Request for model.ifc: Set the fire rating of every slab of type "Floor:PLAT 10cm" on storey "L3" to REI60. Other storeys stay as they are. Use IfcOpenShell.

First a look at what the model holds.

```python
import ifcopenshell
import ifcopenshell.util.element

model = ifcopenshell.open("model.ifc")
print(model.schema)
storey = next(s for s in model.by_type("IfcBuildingStorey") if s.Name == "L3")
slabs = [e for e in ifcopenshell.util.element.get_decomposition(storey) if e.is_a("IfcSlab")]
seen = {}
for e in slabs:
    element_type = ifcopenshell.util.element.get_type(e)
    key = (element_type.Name if element_type != e and element_type else None, ifcopenshell.util.element.get_pset(e, "Pset_SlabCommon", "FireRating"))
    seen[key] = seen.get(key, 0) + 1
for (name, value), count in sorted(seen.items(), key=str):
    print(count, "x", name, "|", value)
```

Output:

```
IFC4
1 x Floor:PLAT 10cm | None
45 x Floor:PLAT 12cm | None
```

```python
import ifcopenshell
import ifcopenshell.api.pset
import ifcopenshell.util.element

model = ifcopenshell.open("model.ifc")

storey = next(s for s in model.by_type("IfcBuildingStorey") if s.Name == "L3")
slabs = [e for e in ifcopenshell.util.element.get_decomposition(storey) if e.is_a("IfcSlab")]

count = 0
for e in slabs:
    element_type = ifcopenshell.util.element.get_type(e)
    if element_type in (None, e) or element_type.Name != "Floor:PLAT 10cm":
        continue
    # add_pset returns the element's existing set when there is one.
    pset = ifcopenshell.api.pset.add_pset(model, product=e, name="Pset_SlabCommon")
    ifcopenshell.api.pset.edit_pset(model, pset=pset, properties={"FireRating": "REI60"})
    count += 1

print(count, "slabs updated")

model.write("model_updated.ifc")
```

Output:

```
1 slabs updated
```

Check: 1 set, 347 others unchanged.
